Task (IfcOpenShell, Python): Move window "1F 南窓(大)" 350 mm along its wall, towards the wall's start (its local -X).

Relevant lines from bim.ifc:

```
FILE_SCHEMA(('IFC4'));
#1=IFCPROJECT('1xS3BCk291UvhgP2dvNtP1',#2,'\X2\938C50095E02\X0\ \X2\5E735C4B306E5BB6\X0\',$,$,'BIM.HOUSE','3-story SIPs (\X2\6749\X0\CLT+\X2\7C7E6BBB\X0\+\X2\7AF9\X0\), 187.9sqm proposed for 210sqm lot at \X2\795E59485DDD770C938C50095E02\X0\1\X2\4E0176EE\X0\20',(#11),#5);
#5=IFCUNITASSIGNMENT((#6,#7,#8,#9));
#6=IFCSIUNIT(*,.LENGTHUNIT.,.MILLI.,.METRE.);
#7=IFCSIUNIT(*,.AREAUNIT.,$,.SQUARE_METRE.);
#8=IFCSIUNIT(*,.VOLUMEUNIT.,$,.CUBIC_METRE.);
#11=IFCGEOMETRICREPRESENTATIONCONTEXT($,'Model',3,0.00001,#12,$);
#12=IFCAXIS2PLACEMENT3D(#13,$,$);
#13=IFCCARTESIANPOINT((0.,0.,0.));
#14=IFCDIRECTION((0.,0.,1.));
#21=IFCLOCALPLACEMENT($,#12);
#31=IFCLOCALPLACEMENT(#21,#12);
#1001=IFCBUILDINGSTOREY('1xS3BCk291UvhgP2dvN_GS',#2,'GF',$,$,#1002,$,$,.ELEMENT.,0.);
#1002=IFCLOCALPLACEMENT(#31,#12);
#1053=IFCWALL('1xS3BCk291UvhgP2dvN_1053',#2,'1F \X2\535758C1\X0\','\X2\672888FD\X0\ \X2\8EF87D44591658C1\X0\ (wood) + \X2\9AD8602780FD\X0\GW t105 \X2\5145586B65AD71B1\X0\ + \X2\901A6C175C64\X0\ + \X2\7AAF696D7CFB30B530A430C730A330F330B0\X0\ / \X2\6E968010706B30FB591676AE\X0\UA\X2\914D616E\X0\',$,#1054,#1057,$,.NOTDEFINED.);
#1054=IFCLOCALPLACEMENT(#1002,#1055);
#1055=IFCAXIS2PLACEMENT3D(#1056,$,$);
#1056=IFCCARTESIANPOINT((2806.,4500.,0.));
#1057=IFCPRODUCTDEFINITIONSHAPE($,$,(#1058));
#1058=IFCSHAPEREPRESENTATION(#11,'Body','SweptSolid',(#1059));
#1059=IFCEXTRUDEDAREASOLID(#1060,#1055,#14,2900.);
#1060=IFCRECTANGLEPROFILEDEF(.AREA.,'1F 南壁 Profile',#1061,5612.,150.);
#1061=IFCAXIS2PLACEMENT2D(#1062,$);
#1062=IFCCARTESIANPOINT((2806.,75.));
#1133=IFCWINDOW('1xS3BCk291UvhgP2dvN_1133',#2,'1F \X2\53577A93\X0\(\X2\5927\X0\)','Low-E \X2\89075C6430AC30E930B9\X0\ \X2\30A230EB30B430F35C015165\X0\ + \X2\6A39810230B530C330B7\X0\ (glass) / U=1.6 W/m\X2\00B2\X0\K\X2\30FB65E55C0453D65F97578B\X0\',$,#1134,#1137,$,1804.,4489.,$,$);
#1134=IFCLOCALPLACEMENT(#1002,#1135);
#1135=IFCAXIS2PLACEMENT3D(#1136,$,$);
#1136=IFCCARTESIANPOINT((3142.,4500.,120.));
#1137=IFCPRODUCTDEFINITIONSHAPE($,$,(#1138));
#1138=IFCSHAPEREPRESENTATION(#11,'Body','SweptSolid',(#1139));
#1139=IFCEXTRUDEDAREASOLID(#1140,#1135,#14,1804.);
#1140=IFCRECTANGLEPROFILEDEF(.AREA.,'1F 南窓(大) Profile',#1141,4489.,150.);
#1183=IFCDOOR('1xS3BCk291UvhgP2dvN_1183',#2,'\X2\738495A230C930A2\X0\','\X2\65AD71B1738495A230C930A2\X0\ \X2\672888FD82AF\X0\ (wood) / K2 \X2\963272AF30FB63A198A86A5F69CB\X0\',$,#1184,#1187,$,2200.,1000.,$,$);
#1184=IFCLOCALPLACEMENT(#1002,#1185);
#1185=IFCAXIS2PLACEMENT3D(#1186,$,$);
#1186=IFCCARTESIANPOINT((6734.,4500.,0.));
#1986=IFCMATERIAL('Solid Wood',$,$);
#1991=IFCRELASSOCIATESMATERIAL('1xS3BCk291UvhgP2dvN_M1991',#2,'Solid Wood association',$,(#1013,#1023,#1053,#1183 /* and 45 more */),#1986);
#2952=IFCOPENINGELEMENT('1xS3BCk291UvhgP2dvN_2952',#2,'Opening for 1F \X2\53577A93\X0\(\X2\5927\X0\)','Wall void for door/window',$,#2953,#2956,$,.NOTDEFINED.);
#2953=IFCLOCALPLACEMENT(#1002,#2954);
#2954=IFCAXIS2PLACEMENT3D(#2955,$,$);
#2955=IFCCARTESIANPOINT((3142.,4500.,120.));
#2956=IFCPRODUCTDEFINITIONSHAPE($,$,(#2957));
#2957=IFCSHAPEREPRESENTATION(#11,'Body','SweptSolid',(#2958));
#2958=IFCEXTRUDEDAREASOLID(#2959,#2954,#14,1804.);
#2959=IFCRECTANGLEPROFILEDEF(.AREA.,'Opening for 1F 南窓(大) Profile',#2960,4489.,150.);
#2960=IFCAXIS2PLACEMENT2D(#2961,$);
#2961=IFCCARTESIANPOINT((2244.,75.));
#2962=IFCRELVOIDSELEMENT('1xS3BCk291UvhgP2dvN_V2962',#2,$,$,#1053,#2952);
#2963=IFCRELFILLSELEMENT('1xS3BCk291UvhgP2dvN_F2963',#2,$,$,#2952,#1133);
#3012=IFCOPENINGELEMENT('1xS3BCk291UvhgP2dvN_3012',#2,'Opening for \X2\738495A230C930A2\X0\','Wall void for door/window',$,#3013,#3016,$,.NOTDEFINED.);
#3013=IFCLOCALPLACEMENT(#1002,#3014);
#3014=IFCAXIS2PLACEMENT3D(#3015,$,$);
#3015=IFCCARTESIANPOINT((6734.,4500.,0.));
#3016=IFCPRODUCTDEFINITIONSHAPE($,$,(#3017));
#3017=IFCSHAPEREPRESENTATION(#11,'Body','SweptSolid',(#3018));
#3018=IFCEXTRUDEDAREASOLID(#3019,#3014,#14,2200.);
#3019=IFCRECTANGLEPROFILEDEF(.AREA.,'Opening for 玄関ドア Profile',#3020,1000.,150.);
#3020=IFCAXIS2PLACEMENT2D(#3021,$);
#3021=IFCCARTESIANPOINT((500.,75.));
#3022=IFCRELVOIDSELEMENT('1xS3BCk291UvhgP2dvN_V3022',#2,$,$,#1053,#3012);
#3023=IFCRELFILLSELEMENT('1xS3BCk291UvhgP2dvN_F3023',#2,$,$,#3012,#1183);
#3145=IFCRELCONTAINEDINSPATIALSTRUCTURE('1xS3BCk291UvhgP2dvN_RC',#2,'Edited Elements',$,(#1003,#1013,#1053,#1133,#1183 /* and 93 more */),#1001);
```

```python
import ifcopenshell
import ifcopenshell.api.geometry
import ifcopenshell.util.placement
import ifcopenshell.util.unit

model = ifcopenshell.open("bim.ifc")
unit_scale = ifcopenshell.util.unit.calculate_unit_scale(model)

window = model.by_id(1133)
opening = window.FillsVoids[0].RelatingOpeningElement
wall = opening.VoidsElements[0].RelatingBuildingElement

wall_matrix = ifcopenshell.util.placement.get_local_placement(wall.ObjectPlacement)
shift = wall_matrix[:3, 0] * -0.35 / unit_scale
before = ifcopenshell.util.placement.get_local_placement(window.ObjectPlacement)[:3, 3].copy()

# The window is not placed relative to its opening, so move both.
for product in (opening, window):
    matrix = ifcopenshell.util.placement.get_local_placement(product.ObjectPlacement)
    matrix[:3, 3] += shift
    ifcopenshell.api.geometry.edit_object_placement(model, product=product, matrix=matrix, is_si=False)

after = ifcopenshell.util.placement.get_local_placement(window.ObjectPlacement)[:3, 3]
print("window moved by", (after - before).round(3) + 0.0)

model.write("bim-out.ifc")
```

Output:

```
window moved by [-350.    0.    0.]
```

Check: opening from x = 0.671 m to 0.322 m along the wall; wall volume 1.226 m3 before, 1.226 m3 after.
